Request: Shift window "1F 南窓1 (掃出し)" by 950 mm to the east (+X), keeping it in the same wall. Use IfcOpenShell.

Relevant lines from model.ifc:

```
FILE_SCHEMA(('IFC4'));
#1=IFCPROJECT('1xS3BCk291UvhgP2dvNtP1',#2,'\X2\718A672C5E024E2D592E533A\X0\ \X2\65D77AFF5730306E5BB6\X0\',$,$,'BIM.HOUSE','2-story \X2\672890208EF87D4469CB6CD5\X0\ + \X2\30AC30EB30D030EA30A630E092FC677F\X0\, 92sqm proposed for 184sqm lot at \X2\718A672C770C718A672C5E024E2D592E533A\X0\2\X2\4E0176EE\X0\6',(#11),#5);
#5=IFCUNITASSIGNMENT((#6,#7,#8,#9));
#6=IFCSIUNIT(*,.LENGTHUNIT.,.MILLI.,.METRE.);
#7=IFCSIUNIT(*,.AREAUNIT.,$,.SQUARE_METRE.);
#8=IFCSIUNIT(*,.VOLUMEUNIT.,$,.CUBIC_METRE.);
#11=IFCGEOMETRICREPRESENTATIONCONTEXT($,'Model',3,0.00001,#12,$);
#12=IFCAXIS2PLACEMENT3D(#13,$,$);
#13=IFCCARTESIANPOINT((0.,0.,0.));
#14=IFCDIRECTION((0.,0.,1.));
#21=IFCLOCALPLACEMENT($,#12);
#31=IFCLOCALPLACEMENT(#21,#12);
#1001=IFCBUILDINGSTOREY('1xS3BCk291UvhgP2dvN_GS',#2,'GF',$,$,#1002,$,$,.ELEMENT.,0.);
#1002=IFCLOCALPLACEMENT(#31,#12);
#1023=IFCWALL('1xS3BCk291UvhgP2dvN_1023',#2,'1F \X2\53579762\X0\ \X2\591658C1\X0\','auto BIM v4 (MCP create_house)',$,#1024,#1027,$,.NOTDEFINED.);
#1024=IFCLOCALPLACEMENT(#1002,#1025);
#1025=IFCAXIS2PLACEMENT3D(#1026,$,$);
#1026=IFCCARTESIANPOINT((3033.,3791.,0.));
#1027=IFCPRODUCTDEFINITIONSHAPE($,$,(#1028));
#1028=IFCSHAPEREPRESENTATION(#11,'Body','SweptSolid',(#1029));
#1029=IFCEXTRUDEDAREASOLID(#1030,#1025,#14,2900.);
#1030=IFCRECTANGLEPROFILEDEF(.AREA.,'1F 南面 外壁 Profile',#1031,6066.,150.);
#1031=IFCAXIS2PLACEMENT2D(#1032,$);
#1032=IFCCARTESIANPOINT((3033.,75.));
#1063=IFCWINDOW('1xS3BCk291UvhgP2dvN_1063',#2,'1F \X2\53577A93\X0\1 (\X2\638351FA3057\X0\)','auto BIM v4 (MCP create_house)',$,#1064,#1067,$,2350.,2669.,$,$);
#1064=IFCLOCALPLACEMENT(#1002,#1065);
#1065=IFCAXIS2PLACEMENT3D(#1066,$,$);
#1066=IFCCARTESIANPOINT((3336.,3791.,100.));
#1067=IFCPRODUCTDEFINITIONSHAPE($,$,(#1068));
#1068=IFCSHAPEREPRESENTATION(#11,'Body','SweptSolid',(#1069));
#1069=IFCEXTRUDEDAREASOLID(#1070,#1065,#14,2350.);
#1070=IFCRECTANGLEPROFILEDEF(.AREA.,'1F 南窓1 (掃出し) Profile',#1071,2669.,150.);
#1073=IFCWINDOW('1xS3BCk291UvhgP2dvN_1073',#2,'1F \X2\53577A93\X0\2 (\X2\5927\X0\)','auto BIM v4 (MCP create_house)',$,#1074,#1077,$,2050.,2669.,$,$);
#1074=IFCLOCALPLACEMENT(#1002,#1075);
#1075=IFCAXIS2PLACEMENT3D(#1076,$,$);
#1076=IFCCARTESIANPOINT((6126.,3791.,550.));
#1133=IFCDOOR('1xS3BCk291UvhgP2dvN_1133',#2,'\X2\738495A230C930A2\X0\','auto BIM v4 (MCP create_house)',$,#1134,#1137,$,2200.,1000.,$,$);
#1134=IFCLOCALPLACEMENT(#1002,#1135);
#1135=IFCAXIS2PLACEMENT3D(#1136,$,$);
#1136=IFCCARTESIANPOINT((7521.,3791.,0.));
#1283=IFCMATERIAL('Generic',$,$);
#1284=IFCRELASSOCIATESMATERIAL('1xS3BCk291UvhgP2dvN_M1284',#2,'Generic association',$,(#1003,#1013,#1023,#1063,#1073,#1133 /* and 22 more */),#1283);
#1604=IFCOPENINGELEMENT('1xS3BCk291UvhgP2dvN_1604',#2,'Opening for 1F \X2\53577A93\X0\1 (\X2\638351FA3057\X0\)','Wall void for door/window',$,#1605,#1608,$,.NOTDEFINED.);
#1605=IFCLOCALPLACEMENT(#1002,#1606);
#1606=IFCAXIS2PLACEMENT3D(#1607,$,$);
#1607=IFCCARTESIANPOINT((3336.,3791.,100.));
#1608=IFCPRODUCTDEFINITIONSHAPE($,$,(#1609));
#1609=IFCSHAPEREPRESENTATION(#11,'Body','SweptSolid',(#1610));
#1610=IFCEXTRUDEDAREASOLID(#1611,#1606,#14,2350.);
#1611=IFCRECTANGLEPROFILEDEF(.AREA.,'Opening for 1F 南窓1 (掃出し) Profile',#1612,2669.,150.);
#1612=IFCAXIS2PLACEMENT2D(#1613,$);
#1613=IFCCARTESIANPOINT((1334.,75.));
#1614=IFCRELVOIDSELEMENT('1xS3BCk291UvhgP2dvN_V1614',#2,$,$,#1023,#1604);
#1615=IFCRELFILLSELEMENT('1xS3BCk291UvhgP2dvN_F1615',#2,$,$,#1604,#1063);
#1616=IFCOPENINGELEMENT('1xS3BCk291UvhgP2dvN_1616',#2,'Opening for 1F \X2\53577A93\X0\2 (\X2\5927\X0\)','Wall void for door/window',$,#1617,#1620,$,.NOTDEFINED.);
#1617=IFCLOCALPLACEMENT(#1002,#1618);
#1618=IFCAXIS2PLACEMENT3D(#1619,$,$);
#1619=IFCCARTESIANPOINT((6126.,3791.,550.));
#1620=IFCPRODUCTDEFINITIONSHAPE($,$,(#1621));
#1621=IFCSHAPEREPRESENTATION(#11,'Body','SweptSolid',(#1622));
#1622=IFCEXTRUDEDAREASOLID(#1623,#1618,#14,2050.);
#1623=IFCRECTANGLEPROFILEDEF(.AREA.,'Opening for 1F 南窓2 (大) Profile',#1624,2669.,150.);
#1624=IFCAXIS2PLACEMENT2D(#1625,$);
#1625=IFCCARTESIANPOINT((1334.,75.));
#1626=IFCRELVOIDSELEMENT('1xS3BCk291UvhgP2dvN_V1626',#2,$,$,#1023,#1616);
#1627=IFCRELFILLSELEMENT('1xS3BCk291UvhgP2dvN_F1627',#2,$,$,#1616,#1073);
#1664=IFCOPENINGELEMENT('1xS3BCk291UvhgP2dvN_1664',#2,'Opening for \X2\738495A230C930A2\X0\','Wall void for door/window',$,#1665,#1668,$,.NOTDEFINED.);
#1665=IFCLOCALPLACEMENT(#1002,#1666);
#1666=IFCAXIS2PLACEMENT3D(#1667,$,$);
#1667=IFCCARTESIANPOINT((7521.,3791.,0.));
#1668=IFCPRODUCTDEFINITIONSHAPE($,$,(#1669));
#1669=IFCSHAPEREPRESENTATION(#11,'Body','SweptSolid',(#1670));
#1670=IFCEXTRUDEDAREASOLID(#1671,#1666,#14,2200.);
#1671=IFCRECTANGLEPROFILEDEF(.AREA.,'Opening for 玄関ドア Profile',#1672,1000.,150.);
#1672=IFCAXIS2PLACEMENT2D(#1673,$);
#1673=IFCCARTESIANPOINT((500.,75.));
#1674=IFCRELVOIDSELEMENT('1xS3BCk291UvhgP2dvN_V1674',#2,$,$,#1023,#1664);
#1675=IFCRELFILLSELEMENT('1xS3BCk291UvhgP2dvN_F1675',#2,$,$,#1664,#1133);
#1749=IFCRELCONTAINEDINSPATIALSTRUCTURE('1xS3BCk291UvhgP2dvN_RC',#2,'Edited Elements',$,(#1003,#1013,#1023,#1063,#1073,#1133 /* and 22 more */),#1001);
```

```python
import ifcopenshell
import ifcopenshell.api.geometry
import ifcopenshell.util.placement
import ifcopenshell.util.unit

model = ifcopenshell.open("model.ifc")
unit_scale = ifcopenshell.util.unit.calculate_unit_scale(model)

window = model.by_id(1063)
opening = window.FillsVoids[0].RelatingOpeningElement
wall = opening.VoidsElements[0].RelatingBuildingElement

wall_matrix = ifcopenshell.util.placement.get_local_placement(wall.ObjectPlacement)
shift = wall_matrix[:3, 0] * 0.95 / unit_scale
before = ifcopenshell.util.placement.get_local_placement(window.ObjectPlacement)[:3, 3].copy()

# The window is not placed relative to its opening, so move both.
for product in (opening, window):
    matrix = ifcopenshell.util.placement.get_local_placement(product.ObjectPlacement)
    matrix[:3, 3] += shift
    ifcopenshell.api.geometry.edit_object_placement(model, product=product, matrix=matrix, is_si=False)

after = ifcopenshell.util.placement.get_local_placement(window.ObjectPlacement)[:3, 3]
print("window moved by", (after - before).round(3) + 0.0)

model.write("model_v2.ifc")
```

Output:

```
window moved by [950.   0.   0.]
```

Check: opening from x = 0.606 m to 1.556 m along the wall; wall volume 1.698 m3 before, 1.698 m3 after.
